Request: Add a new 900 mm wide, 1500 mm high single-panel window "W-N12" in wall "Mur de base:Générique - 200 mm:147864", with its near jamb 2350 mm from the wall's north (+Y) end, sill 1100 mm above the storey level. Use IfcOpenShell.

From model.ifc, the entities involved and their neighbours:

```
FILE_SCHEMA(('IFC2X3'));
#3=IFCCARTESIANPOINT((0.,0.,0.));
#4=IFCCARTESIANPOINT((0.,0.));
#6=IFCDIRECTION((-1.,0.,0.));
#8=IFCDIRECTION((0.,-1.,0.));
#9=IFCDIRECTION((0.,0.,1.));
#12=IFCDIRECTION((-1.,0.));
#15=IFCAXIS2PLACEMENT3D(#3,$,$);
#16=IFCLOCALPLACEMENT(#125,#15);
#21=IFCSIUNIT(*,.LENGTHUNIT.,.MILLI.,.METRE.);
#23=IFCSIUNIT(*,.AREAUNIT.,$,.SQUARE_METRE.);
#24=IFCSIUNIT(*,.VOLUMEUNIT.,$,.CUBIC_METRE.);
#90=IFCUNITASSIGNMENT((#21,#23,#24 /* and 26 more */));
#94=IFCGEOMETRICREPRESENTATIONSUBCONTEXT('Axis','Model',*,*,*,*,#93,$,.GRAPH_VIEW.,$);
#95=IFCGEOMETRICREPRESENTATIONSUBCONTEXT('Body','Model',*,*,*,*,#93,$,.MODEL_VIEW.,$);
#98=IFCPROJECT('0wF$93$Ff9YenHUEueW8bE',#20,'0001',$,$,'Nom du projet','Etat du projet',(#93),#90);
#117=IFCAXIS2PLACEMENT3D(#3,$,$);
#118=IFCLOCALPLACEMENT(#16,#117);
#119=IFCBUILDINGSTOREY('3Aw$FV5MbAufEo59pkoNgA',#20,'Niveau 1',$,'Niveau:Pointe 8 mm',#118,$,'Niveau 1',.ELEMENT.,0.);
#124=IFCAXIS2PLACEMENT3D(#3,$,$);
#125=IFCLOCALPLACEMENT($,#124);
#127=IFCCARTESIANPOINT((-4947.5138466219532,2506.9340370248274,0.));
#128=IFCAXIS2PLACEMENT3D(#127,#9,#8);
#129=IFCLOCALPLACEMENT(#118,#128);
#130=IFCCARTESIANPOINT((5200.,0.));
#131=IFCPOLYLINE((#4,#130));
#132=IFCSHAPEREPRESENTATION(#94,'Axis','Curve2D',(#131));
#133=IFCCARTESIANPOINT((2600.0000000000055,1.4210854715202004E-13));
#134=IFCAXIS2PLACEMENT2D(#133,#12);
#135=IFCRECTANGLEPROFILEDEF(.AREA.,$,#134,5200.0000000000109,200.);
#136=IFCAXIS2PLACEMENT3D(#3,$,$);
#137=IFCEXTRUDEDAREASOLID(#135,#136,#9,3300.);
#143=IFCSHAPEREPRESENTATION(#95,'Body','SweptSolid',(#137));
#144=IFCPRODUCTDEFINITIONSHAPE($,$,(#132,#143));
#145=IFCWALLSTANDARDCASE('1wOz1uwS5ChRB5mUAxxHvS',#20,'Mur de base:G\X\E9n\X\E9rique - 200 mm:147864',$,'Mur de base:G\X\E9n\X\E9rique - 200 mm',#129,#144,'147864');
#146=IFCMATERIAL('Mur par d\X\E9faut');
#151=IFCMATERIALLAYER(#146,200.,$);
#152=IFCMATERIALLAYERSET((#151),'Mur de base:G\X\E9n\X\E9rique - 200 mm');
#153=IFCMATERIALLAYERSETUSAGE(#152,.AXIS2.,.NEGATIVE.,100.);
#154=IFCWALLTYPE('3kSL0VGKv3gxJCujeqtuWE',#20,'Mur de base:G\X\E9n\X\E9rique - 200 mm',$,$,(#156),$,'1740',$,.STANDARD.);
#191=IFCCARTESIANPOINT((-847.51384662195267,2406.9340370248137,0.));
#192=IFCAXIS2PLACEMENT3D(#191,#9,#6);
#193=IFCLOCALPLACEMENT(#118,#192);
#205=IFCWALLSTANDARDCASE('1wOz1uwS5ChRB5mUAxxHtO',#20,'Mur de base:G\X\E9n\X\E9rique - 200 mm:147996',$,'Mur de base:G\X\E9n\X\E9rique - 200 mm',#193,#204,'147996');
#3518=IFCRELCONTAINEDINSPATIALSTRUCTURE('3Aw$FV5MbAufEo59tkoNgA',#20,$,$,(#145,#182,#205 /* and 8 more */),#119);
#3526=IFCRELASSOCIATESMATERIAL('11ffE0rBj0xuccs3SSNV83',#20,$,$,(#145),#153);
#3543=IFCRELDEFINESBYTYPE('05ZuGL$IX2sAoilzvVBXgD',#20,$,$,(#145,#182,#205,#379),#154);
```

```python
import numpy as np
import ifcopenshell
import ifcopenshell.api.feature
import ifcopenshell.api.geometry
import ifcopenshell.api.root
import ifcopenshell.api.spatial
import ifcopenshell.api.type
import ifcopenshell.geom
import ifcopenshell.util.element
import ifcopenshell.util.placement
import ifcopenshell.util.representation
import ifcopenshell.util.shape
import ifcopenshell.util.unit

model = ifcopenshell.open("model.ifc")
unit_scale = ifcopenshell.util.unit.calculate_unit_scale(model)
settings = ifcopenshell.geom.settings()


def volume(element):
    """Net volume in cubic metres, openings subtracted."""
    shape = ifcopenshell.geom.create_shape(settings, element)
    return ifcopenshell.util.shape.get_volume(shape.geometry)


wall = model.by_guid("1wOz1uwS5ChRB5mUAxxHvS")
storey = ifcopenshell.util.element.get_container(wall, ifc_class="IfcBuildingStorey")
context = ifcopenshell.util.representation.get_context(model, "Model", "Body", "MODEL_VIEW")
before = volume(wall)

width, height, from_end, sill = 0.9, 1.5, 2.35, 1.1  # metres

# The wall runs along its own X axis, and the end named is its -X end.
wall_shape = ifcopenshell.geom.create_shape(settings, wall)
x, y, z = ifcopenshell.util.shape.get_vertices(wall_shape.geometry).T
start = x.min() + from_end
face, thickness = float(y.min()), float(y.max() - y.min())
wall_matrix = ifcopenshell.util.placement.get_local_placement(wall.ObjectPlacement)
level = ifcopenshell.util.placement.get_local_placement(storey.ObjectPlacement)[2, 3]


def in_wall(x, y):
    """Placement at x, y metres in the wall's axes, at sill height."""
    matrix = wall_matrix.copy()
    matrix[:, 3] = wall_matrix @ np.array([x / unit_scale, y / unit_scale, 0.0, 1.0])
    matrix[2, 3] = level + sill / unit_scale
    return matrix


# Opening: a box that overshoots both wall faces by 50 mm.
opening = ifcopenshell.api.root.create_entity(model, ifc_class="IfcOpeningElement")
box = ifcopenshell.api.geometry.add_wall_representation(
    model, context=context, length=width, height=height, thickness=thickness + 0.1
)
ifcopenshell.api.geometry.assign_representation(model, product=opening, representation=box)
ifcopenshell.api.geometry.edit_object_placement(model, product=opening, matrix=in_wall(start, face - 0.05), is_si=False)
ifcopenshell.api.feature.add_feature(model, feature=opening, element=wall)

window = ifcopenshell.api.root.create_entity(model, ifc_class="IfcWindow", name="W-N12")
window.OverallWidth, window.OverallHeight = width / unit_scale, height / unit_scale
body = ifcopenshell.api.geometry.add_window_representation(
    model,
    context=context,
    overall_width=window.OverallWidth,
    overall_height=window.OverallHeight,
    partition_type="SINGLE_PANEL",
)
ifcopenshell.api.geometry.assign_representation(model, product=window, representation=body)
ifcopenshell.api.spatial.assign_container(model, products=[window], relating_structure=storey)
fills = ifcopenshell.api.feature.add_filling(model, opening=opening, element=window)
fills.OwnerHistory = window.OwnerHistory  # required in IFC2X3

# IFC2X3 keeps the operation on the window style.
style = ifcopenshell.api.root.create_entity(model, ifc_class="IfcWindowStyle", name="W-N12")
style.OperationType, style.ConstructionType = "SINGLE_PANEL", "NOTDEFINED"
style.ParameterTakesPrecedence = style.Sizeable = False
ifcopenshell.api.type.assign_type(model, related_objects=[window], relating_type=style)

# Centre the window in the wall's thickness.
ifcopenshell.api.geometry.edit_object_placement(model, product=window, matrix=in_wall(start, face), is_si=False)
window_shape = ifcopenshell.geom.create_shape(settings, window)
depth = ifcopenshell.util.shape.get_vertices(window_shape.geometry)[:, 1]
offset = face + thickness / 2 - (depth.min() + depth.max()) / 2
ifcopenshell.api.geometry.edit_object_placement(model, product=window, matrix=in_wall(start, offset), is_si=False)

after = volume(wall)

print(f"wall volume {before:.3f} -> {after:.3f} m3")

model.write("model_rev.ifc")
```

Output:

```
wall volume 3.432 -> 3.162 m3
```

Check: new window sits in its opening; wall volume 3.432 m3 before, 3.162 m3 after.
